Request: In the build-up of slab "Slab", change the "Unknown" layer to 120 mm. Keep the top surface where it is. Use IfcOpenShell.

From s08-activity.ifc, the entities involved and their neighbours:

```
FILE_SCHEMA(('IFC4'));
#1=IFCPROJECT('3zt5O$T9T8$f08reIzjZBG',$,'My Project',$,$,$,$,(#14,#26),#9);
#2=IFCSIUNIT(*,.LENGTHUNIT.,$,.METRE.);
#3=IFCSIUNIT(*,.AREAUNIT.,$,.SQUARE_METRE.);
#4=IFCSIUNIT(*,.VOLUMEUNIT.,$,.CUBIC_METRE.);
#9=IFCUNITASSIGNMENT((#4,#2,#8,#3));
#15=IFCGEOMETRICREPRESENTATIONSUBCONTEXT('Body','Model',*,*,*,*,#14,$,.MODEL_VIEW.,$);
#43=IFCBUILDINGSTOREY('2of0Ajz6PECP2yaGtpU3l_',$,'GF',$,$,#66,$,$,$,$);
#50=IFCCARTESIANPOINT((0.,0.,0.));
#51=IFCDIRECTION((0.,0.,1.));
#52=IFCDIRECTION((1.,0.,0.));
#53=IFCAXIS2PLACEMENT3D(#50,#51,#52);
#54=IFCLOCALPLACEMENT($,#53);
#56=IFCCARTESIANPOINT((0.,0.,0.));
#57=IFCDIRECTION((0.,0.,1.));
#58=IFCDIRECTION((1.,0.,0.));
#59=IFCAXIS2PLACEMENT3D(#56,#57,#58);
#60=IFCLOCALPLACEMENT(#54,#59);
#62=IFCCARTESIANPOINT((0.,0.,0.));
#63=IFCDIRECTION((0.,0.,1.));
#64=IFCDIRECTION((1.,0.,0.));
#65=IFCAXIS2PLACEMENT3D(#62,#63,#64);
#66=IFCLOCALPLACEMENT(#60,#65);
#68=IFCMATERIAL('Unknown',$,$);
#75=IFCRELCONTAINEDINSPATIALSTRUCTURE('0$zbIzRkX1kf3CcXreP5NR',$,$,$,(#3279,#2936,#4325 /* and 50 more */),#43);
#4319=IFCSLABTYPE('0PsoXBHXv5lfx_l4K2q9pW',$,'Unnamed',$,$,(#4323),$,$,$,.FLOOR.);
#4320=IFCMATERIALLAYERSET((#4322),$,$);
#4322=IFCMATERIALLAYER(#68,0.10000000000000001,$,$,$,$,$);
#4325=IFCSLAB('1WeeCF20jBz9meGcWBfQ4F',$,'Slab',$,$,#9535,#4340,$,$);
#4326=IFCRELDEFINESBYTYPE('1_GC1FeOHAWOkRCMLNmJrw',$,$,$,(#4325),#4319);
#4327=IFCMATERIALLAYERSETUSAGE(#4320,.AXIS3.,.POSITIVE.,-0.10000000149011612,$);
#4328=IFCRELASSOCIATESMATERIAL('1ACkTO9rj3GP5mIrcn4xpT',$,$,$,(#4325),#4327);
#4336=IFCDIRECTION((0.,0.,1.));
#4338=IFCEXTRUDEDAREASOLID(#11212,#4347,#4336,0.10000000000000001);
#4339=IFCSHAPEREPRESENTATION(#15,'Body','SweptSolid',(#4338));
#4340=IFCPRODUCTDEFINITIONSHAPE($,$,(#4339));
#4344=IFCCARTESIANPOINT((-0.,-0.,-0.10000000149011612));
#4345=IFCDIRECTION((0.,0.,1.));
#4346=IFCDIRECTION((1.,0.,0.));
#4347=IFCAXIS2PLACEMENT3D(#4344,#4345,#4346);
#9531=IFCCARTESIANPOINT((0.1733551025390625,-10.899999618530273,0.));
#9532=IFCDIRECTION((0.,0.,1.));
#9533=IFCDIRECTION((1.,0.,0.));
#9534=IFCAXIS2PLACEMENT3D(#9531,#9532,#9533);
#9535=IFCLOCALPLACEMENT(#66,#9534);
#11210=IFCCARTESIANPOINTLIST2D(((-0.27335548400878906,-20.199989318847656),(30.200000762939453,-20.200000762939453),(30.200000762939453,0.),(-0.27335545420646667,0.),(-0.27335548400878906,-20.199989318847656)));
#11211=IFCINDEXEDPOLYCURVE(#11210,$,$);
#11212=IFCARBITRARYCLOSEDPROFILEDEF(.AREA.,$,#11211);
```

```python
import ifcopenshell
import ifcopenshell.util.element
import ifcopenshell.util.representation
import ifcopenshell.util.unit

model = ifcopenshell.open("s08-activity.ifc")
unit_scale = ifcopenshell.util.unit.calculate_unit_scale(model)

layer_set = model.by_id(4320)
layer = next(l for l in layer_set.MaterialLayers if l.Material and l.Material.Name == "Unknown")
change = 0.12 / unit_scale - layer.LayerThickness
layer.LayerThickness += change

# Geometry does not follow the layer set by itself.
slabs = [e for e in ifcopenshell.util.element.get_elements_by_material(model, layer_set) if e.is_a("IfcSlab")]
for slab in sorted(slabs, key=lambda e: e.id()):
    body = ifcopenshell.util.representation.get_representation(slab, "Model", "Body")
    solid = body.Items[0]
    old_depth = solid.Depth
    solid.Depth += change
    # Extruded upwards: lower the start of the extrusion so the top stays.
    x, y, z = solid.Position.Location.Coordinates
    solid.Position.Location = model.createIfcCartesianPoint((x, y, z - change))
    print(slab.id(), f"{old_depth:g} -> {solid.Depth:g}")

# The layers are counted up from the underside, which has moved.
for usage in {ifcopenshell.util.element.get_material(slab) for slab in slabs}:
    usage.OffsetFromReferenceLine -= change

model.write("s08-activity_rev.ifc")
```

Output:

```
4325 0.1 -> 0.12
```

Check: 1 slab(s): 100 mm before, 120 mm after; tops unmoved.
